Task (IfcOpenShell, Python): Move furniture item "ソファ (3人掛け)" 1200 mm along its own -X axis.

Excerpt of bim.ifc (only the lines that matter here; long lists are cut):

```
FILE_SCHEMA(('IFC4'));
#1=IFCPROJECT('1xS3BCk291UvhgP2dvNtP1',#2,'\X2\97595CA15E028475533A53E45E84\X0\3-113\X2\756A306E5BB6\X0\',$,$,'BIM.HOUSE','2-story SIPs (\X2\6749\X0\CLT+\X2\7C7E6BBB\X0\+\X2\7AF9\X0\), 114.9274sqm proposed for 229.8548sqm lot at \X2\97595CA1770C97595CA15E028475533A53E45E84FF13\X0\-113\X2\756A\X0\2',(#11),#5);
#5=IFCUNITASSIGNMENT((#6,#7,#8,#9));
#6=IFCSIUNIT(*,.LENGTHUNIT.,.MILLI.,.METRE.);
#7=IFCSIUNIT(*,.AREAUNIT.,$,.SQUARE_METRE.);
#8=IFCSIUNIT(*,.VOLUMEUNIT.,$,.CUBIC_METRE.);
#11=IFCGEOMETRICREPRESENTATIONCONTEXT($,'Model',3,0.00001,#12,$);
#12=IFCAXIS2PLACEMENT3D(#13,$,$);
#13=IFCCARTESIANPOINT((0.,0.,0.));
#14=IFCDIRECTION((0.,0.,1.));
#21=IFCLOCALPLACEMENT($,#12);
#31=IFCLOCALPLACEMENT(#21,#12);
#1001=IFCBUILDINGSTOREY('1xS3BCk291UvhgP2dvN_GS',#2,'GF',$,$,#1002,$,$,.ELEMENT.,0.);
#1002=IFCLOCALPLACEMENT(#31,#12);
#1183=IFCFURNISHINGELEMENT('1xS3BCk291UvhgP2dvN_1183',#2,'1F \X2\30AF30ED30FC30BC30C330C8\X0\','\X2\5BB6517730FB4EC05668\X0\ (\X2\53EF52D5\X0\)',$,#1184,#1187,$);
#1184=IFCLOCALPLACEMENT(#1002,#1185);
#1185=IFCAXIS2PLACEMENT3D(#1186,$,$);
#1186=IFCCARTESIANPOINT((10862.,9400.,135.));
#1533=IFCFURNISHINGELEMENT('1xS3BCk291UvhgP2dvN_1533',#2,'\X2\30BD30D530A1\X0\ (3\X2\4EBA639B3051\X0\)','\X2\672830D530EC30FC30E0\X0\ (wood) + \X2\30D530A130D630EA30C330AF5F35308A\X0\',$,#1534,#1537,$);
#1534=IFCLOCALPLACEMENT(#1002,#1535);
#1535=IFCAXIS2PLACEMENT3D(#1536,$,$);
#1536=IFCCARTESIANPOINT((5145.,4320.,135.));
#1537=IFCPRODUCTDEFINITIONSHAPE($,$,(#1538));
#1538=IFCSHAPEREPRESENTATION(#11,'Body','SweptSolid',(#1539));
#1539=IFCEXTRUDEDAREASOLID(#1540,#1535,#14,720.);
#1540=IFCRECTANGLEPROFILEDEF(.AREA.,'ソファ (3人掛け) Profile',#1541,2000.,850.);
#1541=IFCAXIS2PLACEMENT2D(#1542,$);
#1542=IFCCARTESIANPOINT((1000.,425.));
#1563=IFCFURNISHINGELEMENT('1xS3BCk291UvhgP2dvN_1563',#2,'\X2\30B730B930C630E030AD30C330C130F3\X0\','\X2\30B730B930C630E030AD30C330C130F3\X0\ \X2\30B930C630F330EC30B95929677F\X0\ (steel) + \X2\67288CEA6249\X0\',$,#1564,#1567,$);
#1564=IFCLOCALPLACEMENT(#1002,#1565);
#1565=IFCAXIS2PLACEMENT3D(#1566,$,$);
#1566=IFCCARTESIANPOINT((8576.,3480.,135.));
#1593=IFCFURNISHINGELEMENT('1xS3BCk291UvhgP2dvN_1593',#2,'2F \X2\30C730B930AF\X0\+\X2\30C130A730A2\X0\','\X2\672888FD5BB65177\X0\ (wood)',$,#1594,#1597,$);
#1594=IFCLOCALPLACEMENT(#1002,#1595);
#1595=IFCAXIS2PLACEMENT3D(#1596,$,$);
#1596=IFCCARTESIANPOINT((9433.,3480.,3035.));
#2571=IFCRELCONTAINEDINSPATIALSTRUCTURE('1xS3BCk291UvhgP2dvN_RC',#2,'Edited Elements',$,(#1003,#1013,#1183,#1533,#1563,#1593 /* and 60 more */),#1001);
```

```python
import ifcopenshell
import ifcopenshell.api.geometry
import ifcopenshell.util.placement

model = ifcopenshell.open("bim.ifc")

item = model.by_id(1533)
matrix = ifcopenshell.util.placement.get_local_placement(item.ObjectPlacement)
matrix[:3, 3] -= matrix[:3, 0] * 1200.0
ifcopenshell.api.geometry.edit_object_placement(model, product=item, matrix=matrix, is_si=False)

print(ifcopenshell.util.placement.get_local_placement(item.ObjectPlacement).round(3) + 0.0)

model.write("bim_updated.ifc")
```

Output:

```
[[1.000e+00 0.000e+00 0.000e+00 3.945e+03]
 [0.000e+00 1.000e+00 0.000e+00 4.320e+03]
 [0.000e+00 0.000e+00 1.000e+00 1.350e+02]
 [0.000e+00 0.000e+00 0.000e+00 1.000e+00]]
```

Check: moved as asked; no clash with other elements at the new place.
